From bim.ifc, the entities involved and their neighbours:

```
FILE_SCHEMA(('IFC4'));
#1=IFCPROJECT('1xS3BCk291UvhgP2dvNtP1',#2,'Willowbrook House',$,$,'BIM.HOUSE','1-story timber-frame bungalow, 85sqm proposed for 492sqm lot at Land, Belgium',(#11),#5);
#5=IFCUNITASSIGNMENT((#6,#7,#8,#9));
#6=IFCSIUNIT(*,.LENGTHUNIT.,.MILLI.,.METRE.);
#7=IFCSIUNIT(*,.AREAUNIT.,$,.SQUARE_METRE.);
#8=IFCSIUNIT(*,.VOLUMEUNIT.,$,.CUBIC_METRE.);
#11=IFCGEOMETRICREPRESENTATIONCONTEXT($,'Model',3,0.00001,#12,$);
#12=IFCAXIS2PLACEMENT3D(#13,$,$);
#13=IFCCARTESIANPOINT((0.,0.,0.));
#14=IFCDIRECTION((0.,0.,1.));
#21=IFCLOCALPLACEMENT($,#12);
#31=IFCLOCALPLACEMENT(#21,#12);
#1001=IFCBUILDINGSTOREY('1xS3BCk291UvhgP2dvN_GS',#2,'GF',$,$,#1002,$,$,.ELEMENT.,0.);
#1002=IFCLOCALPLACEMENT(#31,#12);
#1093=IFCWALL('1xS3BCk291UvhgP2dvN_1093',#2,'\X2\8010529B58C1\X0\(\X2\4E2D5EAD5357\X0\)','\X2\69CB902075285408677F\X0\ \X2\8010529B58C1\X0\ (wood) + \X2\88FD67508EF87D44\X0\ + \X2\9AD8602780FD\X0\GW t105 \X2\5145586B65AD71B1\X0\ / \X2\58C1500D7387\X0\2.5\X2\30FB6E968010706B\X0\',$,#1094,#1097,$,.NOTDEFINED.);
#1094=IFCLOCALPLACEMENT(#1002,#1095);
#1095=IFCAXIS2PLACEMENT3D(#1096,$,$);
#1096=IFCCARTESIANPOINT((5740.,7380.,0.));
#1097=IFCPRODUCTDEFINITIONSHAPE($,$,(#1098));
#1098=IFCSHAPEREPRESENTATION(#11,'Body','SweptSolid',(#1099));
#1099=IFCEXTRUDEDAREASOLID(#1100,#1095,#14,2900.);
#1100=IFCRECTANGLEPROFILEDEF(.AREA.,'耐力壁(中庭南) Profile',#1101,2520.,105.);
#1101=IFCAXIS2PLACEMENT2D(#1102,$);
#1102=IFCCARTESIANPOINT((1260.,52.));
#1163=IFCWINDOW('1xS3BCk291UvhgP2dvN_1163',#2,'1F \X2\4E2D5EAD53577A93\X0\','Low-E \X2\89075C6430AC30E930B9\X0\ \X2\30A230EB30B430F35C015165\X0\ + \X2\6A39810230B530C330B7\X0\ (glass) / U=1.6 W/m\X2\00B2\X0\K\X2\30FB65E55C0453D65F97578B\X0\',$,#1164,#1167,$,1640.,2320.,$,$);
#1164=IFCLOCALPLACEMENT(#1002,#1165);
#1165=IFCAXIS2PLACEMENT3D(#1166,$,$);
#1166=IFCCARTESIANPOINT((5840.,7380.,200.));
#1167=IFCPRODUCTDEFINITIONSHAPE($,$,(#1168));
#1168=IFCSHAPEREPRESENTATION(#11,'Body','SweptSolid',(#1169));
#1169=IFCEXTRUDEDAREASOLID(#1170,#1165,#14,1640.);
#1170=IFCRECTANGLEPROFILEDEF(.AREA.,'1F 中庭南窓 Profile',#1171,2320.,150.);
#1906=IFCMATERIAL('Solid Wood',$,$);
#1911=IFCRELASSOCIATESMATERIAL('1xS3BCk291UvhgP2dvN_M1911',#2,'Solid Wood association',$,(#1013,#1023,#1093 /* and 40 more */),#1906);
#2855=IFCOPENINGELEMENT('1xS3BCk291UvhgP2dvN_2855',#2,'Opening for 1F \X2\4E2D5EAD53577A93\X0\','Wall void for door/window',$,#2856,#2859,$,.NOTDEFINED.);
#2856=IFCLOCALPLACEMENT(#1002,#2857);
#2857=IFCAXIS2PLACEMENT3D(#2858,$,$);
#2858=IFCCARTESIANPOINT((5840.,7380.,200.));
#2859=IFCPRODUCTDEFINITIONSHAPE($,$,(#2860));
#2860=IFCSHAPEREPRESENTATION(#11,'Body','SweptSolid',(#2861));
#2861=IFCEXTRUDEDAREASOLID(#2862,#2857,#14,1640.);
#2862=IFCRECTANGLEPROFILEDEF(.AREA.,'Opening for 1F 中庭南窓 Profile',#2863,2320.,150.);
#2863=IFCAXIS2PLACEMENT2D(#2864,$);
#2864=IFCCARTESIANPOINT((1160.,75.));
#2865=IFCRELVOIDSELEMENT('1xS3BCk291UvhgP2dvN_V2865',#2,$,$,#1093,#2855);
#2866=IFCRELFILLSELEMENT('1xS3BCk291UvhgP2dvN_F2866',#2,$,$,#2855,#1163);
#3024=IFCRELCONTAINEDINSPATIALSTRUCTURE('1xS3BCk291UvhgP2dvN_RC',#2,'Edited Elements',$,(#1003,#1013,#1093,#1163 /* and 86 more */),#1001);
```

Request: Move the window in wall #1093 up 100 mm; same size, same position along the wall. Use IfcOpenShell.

```python
import numpy as np
import ifcopenshell
import ifcopenshell.api.geometry
import ifcopenshell.util.placement
import ifcopenshell.util.unit

model = ifcopenshell.open("bim.ifc")
unit_scale = ifcopenshell.util.unit.calculate_unit_scale(model)

window = model.by_guid("1xS3BCk291UvhgP2dvN_1163")
opening = window.FillsVoids[0].RelatingOpeningElement
dz = 0.1 / unit_scale

shift = np.array([0.0, 0.0, dz])
# The window is not placed relative to its opening, so move both.
for product in (opening, window):
    matrix = ifcopenshell.util.placement.get_local_placement(product.ObjectPlacement)
    matrix[:3, 3] += shift
    ifcopenshell.api.geometry.edit_object_placement(model, product=product, matrix=matrix, is_si=False)

print(f"moved by {dz * unit_scale:+.3f} m")

model.write("bim_v2.ifc")
```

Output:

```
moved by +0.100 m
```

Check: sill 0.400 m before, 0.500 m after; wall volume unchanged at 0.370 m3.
